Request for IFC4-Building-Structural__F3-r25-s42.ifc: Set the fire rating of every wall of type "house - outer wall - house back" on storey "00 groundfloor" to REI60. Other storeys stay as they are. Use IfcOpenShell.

First a look at what the model holds.

```python
import ifcopenshell
import ifcopenshell.util.element

model = ifcopenshell.open("IFC4-Building-Structural__F3-r25-s42.ifc")
print(model.schema)
storey = next(s for s in model.by_type("IfcBuildingStorey") if s.Name == "00 groundfloor")
walls = [e for e in ifcopenshell.util.element.get_decomposition(storey) if e.is_a("IfcWall")]
seen = {}
for e in walls:
    element_type = ifcopenshell.util.element.get_type(e)
    key = (element_type.Name if element_type != e and element_type else None, ifcopenshell.util.element.get_pset(e, "Pset_WallCommon", "FireRating"))
    seen[key] = seen.get(key, 0) + 1
for (name, value), count in sorted(seen.items(), key=str):
    print(count, "x", name, "|", value)
```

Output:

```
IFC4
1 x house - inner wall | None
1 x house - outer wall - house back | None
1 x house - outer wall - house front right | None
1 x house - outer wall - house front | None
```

```python
import ifcopenshell
import ifcopenshell.api.pset
import ifcopenshell.util.element

model = ifcopenshell.open("IFC4-Building-Structural__F3-r25-s42.ifc")

storey = next(s for s in model.by_type("IfcBuildingStorey") if s.Name == "00 groundfloor")
walls = [e for e in ifcopenshell.util.element.get_decomposition(storey) if e.is_a("IfcWall")]

count = 0
for e in walls:
    element_type = ifcopenshell.util.element.get_type(e)
    if element_type in (None, e) or element_type.Name != "house - outer wall - house back":
        continue
    # add_pset returns the element's existing set when there is one.
    pset = ifcopenshell.api.pset.add_pset(model, product=e, name="Pset_WallCommon")
    ifcopenshell.api.pset.edit_pset(model, pset=pset, properties={"FireRating": "REI60"})
    count += 1

print(count, "walls updated")

model.write("IFC4-Building-Structural__F3-r25-s42_v2.ifc")
```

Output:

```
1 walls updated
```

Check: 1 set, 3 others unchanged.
